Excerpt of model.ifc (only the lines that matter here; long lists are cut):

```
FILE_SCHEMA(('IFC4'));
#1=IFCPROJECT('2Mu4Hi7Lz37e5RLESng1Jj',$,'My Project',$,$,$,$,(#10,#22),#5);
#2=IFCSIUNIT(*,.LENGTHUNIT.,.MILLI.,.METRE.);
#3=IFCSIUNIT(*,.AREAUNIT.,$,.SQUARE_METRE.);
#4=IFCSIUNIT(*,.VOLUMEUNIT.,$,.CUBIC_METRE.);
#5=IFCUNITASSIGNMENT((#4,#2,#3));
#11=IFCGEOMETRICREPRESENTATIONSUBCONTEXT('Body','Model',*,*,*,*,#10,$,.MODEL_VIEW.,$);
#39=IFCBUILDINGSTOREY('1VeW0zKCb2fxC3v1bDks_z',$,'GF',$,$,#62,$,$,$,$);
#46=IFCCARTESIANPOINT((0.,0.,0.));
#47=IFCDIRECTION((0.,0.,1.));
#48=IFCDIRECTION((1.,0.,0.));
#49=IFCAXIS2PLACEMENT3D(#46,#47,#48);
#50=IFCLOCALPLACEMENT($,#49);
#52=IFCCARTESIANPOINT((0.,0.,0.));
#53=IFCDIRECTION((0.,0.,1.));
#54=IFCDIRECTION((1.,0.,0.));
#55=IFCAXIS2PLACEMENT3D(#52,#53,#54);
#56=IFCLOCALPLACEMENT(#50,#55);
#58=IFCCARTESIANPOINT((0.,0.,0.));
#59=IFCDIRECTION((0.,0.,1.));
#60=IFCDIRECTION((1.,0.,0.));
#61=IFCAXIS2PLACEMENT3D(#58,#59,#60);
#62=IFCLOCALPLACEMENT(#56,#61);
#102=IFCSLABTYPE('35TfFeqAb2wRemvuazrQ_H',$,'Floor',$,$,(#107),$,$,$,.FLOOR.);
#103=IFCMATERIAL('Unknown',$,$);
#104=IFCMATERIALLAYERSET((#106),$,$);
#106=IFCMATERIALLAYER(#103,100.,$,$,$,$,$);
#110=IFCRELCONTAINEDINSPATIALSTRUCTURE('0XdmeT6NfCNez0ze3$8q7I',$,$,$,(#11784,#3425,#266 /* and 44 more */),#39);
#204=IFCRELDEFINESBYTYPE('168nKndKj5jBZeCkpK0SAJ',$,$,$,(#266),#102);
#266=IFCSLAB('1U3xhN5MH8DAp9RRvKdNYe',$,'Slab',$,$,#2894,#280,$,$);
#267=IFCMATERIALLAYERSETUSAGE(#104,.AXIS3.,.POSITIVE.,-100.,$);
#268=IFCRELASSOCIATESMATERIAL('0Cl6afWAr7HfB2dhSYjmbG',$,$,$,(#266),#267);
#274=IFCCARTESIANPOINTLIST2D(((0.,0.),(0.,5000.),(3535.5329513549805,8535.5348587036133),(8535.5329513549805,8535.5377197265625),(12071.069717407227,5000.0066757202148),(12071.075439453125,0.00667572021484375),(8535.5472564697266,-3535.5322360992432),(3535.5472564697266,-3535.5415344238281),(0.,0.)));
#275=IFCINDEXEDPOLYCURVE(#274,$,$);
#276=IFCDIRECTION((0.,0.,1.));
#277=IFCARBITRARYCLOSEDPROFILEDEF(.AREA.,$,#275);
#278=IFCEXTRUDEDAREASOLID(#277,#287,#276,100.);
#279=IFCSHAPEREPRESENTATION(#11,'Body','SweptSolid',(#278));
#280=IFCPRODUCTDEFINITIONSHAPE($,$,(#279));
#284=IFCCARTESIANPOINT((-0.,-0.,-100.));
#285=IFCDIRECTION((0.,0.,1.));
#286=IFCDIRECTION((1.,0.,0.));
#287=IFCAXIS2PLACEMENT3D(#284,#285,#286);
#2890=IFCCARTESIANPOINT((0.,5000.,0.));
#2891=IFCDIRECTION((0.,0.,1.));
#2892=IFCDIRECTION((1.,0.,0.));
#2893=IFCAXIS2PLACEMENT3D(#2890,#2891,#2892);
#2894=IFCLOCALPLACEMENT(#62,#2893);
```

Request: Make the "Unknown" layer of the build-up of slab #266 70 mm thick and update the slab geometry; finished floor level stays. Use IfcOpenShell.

```python
import ifcopenshell
import ifcopenshell.util.element
import ifcopenshell.util.representation
import ifcopenshell.util.unit

model = ifcopenshell.open("model.ifc")
unit_scale = ifcopenshell.util.unit.calculate_unit_scale(model)

layer_set = model.by_id(104)
layer = next(l for l in layer_set.MaterialLayers if l.Material and l.Material.Name == "Unknown")
change = 0.07 / unit_scale - layer.LayerThickness
layer.LayerThickness += change

# Geometry does not follow the layer set by itself.
slabs = [e for e in ifcopenshell.util.element.get_elements_by_material(model, layer_set) if e.is_a("IfcSlab")]
for slab in sorted(slabs, key=lambda e: e.id()):
    body = ifcopenshell.util.representation.get_representation(slab, "Model", "Body")
    solid = body.Items[0]
    old_depth = solid.Depth
    solid.Depth += change
    # Extruded upwards: lower the start of the extrusion so the top stays.
    x, y, z = solid.Position.Location.Coordinates
    solid.Position.Location = model.createIfcCartesianPoint((x, y, z - change))
    print(slab.id(), f"{old_depth:g} -> {solid.Depth:g}")

# The layers are counted up from the underside, which has moved.
for usage in {ifcopenshell.util.element.get_material(slab) for slab in slabs}:
    usage.OffsetFromReferenceLine -= change

model.write("model_edited.ifc")
```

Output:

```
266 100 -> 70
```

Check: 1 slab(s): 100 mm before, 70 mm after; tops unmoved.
